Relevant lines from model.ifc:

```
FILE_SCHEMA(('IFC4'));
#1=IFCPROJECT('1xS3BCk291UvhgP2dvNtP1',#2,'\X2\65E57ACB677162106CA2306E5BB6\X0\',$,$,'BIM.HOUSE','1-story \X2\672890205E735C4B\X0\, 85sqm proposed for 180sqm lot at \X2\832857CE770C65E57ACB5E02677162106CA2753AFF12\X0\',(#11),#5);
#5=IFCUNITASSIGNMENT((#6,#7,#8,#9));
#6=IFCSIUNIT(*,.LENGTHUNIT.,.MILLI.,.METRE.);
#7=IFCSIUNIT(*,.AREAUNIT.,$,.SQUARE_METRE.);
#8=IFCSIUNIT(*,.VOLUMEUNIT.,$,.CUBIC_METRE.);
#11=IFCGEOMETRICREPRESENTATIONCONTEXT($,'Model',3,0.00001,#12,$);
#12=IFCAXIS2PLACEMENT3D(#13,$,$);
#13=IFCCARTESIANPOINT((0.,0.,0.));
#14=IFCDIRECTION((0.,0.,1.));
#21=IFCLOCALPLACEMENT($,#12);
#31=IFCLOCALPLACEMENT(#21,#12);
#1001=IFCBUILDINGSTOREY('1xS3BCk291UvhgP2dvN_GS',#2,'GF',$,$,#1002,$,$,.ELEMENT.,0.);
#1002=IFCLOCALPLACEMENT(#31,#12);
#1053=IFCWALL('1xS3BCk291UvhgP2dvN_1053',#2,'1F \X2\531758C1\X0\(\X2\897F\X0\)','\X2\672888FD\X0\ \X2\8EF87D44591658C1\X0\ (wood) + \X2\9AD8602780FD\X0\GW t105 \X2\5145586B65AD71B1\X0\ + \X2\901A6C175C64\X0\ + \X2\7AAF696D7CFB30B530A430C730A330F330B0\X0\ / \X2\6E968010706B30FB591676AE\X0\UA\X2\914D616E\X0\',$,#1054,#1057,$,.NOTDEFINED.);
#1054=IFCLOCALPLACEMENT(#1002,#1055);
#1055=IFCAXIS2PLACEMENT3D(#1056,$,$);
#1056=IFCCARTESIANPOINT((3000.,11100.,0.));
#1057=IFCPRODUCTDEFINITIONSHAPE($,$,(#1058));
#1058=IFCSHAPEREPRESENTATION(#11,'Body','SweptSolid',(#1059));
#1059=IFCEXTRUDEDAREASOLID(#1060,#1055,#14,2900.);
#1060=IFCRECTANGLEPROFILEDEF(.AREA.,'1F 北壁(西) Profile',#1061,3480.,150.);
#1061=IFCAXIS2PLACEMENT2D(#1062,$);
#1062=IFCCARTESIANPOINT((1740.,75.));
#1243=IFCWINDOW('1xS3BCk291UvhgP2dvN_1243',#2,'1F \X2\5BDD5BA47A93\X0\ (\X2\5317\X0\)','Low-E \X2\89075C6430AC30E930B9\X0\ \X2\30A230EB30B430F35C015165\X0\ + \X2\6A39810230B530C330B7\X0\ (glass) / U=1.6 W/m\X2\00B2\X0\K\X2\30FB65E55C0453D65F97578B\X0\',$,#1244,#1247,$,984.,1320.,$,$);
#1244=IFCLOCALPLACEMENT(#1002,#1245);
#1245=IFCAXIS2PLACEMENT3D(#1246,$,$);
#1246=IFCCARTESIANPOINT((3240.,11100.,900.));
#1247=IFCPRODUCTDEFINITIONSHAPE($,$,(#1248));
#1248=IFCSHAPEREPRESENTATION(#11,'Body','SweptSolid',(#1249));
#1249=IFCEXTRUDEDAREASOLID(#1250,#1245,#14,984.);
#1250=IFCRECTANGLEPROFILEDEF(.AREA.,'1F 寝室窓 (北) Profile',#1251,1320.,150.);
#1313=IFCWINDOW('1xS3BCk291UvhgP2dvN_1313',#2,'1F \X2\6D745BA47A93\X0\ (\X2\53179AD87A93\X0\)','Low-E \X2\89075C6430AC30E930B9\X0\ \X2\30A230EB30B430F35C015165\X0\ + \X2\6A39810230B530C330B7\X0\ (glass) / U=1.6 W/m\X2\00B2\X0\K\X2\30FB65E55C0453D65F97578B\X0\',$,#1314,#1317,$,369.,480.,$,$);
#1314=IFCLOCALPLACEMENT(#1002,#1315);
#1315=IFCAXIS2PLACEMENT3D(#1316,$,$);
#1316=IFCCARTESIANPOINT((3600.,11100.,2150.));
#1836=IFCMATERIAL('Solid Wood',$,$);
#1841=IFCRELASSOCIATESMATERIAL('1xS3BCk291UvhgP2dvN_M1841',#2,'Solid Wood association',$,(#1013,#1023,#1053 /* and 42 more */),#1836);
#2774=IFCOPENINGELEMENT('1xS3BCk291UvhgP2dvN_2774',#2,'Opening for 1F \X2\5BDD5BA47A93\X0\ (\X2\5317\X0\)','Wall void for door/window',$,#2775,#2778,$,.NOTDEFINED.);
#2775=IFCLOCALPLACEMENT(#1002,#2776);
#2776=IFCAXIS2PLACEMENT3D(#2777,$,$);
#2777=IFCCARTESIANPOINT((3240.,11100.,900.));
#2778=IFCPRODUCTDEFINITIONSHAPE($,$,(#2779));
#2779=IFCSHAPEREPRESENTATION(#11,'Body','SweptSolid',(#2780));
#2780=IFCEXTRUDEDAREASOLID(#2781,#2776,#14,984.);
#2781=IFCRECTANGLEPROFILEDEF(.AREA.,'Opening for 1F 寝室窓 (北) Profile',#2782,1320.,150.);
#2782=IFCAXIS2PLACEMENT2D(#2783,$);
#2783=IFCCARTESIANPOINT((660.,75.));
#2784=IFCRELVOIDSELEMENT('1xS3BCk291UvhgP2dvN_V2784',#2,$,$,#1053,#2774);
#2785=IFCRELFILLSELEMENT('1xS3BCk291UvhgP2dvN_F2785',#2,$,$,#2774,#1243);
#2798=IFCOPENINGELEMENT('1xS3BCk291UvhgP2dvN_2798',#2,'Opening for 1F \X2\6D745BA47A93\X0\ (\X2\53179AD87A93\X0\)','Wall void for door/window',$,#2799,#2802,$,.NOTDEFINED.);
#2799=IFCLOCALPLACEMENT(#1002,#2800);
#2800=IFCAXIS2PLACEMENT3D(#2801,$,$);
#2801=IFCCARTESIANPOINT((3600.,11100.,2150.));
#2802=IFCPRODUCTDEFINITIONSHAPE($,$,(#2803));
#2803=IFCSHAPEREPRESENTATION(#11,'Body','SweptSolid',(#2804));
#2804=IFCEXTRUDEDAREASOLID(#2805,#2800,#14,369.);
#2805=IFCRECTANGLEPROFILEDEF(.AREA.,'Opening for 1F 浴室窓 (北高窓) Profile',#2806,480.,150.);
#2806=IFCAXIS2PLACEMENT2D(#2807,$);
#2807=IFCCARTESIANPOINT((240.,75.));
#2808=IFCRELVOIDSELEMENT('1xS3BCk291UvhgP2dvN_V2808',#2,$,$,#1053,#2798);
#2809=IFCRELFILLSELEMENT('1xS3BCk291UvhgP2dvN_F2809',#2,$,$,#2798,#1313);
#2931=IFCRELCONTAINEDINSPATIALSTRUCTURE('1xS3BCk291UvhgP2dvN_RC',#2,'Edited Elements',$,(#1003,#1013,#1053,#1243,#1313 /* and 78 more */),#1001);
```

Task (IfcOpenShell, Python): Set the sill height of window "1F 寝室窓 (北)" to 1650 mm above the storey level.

```python
import numpy as np
import ifcopenshell
import ifcopenshell.api.geometry
import ifcopenshell.geom
import ifcopenshell.util.element
import ifcopenshell.util.placement
import ifcopenshell.util.shape
import ifcopenshell.util.unit

model = ifcopenshell.open("model.ifc")
unit_scale = ifcopenshell.util.unit.calculate_unit_scale(model)

window = model.by_guid("1xS3BCk291UvhgP2dvN_1243")
opening = window.FillsVoids[0].RelatingOpeningElement
storey = ifcopenshell.util.element.get_container(window, ifc_class="IfcBuildingStorey")
level = ifcopenshell.util.placement.get_local_placement(storey.ObjectPlacement)[2, 3]

# The opening's origin need not be at the sill, so measure its lowest point.
shape = ifcopenshell.geom.create_shape(ifcopenshell.geom.settings(), opening)
bottom = ifcopenshell.util.shape.get_shape_bottom_elevation(shape, shape.geometry) / unit_scale
dz = level + 1650.0 - bottom

shift = np.array([0.0, 0.0, dz])
# The window is not placed relative to its opening, so move both.
for product in (opening, window):
    matrix = ifcopenshell.util.placement.get_local_placement(product.ObjectPlacement)
    matrix[:3, 3] += shift
    ifcopenshell.api.geometry.edit_object_placement(model, product=product, matrix=matrix, is_si=False)

print(f"moved by {dz * unit_scale:+.3f} m")

model.write("model_rev.ifc")
```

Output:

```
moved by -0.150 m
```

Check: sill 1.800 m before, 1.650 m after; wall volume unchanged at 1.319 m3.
